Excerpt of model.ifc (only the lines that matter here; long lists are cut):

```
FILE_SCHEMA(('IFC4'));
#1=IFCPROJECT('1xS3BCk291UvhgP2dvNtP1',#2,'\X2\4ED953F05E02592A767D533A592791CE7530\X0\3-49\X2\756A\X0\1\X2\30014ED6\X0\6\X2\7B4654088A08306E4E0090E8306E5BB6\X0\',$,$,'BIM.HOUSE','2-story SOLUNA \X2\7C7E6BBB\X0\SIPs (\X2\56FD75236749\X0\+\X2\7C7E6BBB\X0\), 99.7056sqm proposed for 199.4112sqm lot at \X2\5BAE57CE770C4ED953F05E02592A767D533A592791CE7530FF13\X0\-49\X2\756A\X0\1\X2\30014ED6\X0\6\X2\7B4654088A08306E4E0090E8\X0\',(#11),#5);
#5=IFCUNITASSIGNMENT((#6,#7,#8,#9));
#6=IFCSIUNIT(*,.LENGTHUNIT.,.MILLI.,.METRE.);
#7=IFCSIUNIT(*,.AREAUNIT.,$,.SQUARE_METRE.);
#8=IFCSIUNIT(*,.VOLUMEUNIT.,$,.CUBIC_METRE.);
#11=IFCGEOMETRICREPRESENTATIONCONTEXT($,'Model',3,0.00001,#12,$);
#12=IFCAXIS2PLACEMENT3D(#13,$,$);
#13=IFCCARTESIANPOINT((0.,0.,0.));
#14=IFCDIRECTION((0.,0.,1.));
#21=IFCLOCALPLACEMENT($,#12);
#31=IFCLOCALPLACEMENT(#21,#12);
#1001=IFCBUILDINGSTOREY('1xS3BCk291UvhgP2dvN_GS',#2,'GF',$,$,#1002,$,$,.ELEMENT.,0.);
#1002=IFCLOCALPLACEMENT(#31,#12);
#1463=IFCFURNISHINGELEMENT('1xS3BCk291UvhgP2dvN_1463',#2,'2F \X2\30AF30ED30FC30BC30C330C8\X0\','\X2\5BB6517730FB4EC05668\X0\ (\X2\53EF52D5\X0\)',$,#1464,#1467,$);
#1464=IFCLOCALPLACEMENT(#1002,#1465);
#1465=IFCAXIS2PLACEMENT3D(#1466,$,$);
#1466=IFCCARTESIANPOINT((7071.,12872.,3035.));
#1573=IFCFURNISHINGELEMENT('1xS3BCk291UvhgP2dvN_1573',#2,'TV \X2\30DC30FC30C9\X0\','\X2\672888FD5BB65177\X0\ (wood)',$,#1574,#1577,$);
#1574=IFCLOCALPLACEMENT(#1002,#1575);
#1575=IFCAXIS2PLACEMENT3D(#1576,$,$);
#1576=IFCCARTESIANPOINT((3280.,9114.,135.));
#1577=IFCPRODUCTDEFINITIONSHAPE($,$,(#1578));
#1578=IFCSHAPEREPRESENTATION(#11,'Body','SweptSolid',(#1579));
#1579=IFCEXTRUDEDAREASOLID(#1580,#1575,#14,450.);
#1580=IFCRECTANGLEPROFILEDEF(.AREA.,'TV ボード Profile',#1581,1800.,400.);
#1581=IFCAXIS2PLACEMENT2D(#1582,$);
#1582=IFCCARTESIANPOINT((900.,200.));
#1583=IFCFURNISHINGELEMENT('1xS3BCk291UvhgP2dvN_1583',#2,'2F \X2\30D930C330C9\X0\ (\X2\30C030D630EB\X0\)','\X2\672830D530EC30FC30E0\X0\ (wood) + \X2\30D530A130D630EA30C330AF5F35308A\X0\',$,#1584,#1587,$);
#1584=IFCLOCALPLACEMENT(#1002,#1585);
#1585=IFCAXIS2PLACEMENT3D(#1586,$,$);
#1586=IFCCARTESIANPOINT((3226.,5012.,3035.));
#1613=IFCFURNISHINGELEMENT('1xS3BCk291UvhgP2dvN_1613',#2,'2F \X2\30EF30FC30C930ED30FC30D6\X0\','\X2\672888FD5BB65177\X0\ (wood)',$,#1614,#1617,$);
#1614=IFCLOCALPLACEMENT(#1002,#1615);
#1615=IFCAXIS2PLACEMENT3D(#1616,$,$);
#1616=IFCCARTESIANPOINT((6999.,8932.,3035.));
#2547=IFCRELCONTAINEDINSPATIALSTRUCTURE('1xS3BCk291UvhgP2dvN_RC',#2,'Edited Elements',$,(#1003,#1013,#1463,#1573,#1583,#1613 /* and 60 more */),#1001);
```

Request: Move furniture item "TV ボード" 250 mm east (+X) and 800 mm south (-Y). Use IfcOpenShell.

```python
import ifcopenshell
import ifcopenshell.api.geometry
import ifcopenshell.util.placement
import ifcopenshell.util.unit

model = ifcopenshell.open("model.ifc")
unit_scale = ifcopenshell.util.unit.calculate_unit_scale(model)

item = model.by_id(1573)
matrix = ifcopenshell.util.placement.get_local_placement(item.ObjectPlacement)
matrix[0, 3] += 0.25 / unit_scale
matrix[1, 3] -= 0.8 / unit_scale
ifcopenshell.api.geometry.edit_object_placement(model, product=item, matrix=matrix, is_si=False)

print(ifcopenshell.util.placement.get_local_placement(item.ObjectPlacement).round(3) + 0.0)

model.write("model_rev.ifc")
```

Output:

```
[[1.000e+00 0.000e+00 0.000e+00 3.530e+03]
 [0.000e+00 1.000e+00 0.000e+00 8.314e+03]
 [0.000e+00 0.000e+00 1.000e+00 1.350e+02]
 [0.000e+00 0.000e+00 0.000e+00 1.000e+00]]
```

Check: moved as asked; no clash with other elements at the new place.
